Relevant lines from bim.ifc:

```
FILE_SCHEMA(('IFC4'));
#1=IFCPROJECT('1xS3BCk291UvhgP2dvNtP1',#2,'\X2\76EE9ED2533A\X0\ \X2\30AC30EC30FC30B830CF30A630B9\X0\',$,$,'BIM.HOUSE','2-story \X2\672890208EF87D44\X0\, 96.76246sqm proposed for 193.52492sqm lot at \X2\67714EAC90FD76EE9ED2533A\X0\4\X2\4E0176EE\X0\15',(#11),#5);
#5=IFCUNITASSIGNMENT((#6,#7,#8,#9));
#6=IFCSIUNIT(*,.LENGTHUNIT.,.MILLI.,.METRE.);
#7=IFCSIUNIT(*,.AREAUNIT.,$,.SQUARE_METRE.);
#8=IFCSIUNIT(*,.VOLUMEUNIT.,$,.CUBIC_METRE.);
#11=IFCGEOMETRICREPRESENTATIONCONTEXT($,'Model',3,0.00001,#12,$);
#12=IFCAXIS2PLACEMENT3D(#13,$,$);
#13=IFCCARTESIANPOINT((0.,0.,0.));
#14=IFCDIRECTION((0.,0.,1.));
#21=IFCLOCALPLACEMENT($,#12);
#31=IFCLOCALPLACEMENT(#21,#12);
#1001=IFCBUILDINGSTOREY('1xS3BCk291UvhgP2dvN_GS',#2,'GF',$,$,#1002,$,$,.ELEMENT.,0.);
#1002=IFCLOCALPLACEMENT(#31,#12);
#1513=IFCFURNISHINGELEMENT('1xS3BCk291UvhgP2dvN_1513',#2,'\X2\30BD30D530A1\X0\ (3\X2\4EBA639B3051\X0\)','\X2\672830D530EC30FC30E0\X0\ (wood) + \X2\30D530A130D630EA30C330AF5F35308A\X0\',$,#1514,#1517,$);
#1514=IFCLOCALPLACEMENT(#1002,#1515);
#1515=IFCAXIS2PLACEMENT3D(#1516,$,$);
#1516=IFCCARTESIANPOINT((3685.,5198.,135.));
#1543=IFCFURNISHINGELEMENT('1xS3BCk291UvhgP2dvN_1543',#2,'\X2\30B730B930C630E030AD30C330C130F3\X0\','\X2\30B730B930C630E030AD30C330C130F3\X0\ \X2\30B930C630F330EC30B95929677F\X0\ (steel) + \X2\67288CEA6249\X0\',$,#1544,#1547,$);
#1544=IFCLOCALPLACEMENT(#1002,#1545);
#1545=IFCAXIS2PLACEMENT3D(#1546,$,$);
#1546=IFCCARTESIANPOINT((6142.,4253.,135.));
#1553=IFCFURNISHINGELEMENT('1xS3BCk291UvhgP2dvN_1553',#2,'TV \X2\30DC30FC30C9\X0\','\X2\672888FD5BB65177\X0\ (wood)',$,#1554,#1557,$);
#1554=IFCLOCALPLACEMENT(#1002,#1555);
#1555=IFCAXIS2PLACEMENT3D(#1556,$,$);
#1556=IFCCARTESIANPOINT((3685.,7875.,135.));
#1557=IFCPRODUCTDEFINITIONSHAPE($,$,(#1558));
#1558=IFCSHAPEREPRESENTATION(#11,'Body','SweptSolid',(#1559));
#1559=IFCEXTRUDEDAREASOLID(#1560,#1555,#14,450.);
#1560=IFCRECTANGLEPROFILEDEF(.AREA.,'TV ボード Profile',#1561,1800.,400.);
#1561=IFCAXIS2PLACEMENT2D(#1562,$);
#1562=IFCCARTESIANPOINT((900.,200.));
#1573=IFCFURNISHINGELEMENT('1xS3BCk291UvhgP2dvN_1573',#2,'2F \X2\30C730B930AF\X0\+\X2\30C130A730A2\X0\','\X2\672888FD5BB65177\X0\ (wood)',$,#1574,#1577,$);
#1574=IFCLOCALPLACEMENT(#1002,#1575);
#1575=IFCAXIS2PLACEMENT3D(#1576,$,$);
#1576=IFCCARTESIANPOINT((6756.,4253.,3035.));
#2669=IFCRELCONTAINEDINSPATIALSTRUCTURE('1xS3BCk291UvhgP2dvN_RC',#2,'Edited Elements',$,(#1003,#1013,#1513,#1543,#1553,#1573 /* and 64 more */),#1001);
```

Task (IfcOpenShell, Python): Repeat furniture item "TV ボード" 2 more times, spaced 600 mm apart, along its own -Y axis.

```python
import ifcopenshell
import ifcopenshell.api.geometry
import ifcopenshell.api.root
import ifcopenshell.util.element
import ifcopenshell.util.placement
import ifcopenshell.util.unit

model = ifcopenshell.open("bim.ifc")
unit_scale = ifcopenshell.util.unit.calculate_unit_scale(model)


def reuse_history(source, copy):
    """copy_class also copies each property set's owner history, people and application; keep the originals."""
    for rel in copy.IsDefinedBy:
        if rel.is_a("IfcRelDefinesByProperties") and (history := rel.RelatingPropertyDefinition.OwnerHistory):
            rel.RelatingPropertyDefinition.OwnerHistory = source.OwnerHistory
            ifcopenshell.util.element.remove_deep2(model, history)


source = model.by_id(1553)
base = ifcopenshell.util.placement.get_local_placement(source.ObjectPlacement)
step = -base[:3, 1] * 0.6 / unit_scale

for i in range(1, 3):
    copy = ifcopenshell.api.root.copy_class(model, product=source)
    copy.Representation = ifcopenshell.util.element.copy_deep(
        model, source.Representation, exclude=["IfcGeometricRepresentationContext", "IfcRepresentationMap"]
    )
    reuse_history(source, copy)
    matrix = base.copy()
    matrix[:3, 3] += i * step
    print("added at", matrix[:3, 3].round(3) + 0.0)
    ifcopenshell.api.geometry.edit_object_placement(model, product=copy, matrix=matrix, is_si=False)

model.write("bim_updated.ifc")
```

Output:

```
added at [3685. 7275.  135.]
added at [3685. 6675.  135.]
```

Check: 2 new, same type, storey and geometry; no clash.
